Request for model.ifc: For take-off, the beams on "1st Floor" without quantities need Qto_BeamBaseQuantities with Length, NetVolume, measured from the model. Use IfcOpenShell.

First a look at what the model holds.

```python
import ifcopenshell
import ifcopenshell.util.element
import ifcopenshell.util.unit

model = ifcopenshell.open("model.ifc")
print(model.schema)
for unit_type in ("LENGTHUNIT", "AREAUNIT", "VOLUMEUNIT"):
    print(unit_type, ifcopenshell.util.unit.calculate_unit_scale(model, unit_type))
storey = next(s for s in model.by_type("IfcBuildingStorey") if s.Name == "1st Floor")
beams = [e for e in ifcopenshell.util.element.get_decomposition(storey) if e.is_a("IfcBeam")]
for e in sorted(beams, key=lambda e: e.id()):
    print(e.id(), e.is_a(), e.Name, list(ifcopenshell.util.element.get_psets(e, qtos_only=True)), sep=" | ")
```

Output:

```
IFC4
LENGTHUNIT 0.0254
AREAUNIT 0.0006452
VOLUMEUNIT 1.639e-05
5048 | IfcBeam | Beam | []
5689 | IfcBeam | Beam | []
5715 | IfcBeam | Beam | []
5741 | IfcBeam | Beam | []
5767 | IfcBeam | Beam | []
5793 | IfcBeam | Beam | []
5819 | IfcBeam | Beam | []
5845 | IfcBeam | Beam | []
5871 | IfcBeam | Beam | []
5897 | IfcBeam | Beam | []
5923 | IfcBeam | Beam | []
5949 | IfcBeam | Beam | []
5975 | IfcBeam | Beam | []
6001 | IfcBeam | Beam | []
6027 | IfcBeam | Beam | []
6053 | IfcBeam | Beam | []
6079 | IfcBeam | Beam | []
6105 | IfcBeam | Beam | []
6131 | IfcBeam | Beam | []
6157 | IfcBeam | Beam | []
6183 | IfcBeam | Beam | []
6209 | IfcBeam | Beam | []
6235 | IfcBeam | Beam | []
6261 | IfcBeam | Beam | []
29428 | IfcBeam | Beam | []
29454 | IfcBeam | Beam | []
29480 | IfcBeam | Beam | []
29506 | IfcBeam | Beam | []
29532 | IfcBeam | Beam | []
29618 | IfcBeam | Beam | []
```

```python
import ifcopenshell
import ifcopenshell.api.pset
import ifcopenshell.geom
import ifcopenshell.util.element
import ifcopenshell.util.shape
import ifcopenshell.util.unit

model = ifcopenshell.open("model.ifc")
unit_scale = ifcopenshell.util.unit.calculate_unit_scale(model)
volume_scale = ifcopenshell.util.unit.calculate_unit_scale(model, "VOLUMEUNIT")
settings = ifcopenshell.geom.settings()

storey = next(s for s in model.by_type("IfcBuildingStorey") if s.Name == "1st Floor")
beams = [e for e in ifcopenshell.util.element.get_decomposition(storey) if e.is_a("IfcBeam")]

for e in sorted(beams, key=lambda e: e.id()):
    if ifcopenshell.util.element.get_psets(e, qtos_only=True, should_inherit=False):
        continue
    # Geometry comes back in metres, in the element's own axes.
    shape = ifcopenshell.geom.create_shape(settings, e)
    values = {
        "Length": ifcopenshell.util.shape.get_max_xyz(shape.geometry) / unit_scale,
        "NetVolume": ifcopenshell.util.shape.get_volume(shape.geometry) / volume_scale,
    }
    qto = ifcopenshell.api.pset.add_qto(model, product=e, name="Qto_BeamBaseQuantities")
    ifcopenshell.api.pset.edit_qto(model, qto=qto, properties=values)
    print(e.id(), {k: round(v, 3) for k, v in values.items()})

model.write("model_v2.ifc")
```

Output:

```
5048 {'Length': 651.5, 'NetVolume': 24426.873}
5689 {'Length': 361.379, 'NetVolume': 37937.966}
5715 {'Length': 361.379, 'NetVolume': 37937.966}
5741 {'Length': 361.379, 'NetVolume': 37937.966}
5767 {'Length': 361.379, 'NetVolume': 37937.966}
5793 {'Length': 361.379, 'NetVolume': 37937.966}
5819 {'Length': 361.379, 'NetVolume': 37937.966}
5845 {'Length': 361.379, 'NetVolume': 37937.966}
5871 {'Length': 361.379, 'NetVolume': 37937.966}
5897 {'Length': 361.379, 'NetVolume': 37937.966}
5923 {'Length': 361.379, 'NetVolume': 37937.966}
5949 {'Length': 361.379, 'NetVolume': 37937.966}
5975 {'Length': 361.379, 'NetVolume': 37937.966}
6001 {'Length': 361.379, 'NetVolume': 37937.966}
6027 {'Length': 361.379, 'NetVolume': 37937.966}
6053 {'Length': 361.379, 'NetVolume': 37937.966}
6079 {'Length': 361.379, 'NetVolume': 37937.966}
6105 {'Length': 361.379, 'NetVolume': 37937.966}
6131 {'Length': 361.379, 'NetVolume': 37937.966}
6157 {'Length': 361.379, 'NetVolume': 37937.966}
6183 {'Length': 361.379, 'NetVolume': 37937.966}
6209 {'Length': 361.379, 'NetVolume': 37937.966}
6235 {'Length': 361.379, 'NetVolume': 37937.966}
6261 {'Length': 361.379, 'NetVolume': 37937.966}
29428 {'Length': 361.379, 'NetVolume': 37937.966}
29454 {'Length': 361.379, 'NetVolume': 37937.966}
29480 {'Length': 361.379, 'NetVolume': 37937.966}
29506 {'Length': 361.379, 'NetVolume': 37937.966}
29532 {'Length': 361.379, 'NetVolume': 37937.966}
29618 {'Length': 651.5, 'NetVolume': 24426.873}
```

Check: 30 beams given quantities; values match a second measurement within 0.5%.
